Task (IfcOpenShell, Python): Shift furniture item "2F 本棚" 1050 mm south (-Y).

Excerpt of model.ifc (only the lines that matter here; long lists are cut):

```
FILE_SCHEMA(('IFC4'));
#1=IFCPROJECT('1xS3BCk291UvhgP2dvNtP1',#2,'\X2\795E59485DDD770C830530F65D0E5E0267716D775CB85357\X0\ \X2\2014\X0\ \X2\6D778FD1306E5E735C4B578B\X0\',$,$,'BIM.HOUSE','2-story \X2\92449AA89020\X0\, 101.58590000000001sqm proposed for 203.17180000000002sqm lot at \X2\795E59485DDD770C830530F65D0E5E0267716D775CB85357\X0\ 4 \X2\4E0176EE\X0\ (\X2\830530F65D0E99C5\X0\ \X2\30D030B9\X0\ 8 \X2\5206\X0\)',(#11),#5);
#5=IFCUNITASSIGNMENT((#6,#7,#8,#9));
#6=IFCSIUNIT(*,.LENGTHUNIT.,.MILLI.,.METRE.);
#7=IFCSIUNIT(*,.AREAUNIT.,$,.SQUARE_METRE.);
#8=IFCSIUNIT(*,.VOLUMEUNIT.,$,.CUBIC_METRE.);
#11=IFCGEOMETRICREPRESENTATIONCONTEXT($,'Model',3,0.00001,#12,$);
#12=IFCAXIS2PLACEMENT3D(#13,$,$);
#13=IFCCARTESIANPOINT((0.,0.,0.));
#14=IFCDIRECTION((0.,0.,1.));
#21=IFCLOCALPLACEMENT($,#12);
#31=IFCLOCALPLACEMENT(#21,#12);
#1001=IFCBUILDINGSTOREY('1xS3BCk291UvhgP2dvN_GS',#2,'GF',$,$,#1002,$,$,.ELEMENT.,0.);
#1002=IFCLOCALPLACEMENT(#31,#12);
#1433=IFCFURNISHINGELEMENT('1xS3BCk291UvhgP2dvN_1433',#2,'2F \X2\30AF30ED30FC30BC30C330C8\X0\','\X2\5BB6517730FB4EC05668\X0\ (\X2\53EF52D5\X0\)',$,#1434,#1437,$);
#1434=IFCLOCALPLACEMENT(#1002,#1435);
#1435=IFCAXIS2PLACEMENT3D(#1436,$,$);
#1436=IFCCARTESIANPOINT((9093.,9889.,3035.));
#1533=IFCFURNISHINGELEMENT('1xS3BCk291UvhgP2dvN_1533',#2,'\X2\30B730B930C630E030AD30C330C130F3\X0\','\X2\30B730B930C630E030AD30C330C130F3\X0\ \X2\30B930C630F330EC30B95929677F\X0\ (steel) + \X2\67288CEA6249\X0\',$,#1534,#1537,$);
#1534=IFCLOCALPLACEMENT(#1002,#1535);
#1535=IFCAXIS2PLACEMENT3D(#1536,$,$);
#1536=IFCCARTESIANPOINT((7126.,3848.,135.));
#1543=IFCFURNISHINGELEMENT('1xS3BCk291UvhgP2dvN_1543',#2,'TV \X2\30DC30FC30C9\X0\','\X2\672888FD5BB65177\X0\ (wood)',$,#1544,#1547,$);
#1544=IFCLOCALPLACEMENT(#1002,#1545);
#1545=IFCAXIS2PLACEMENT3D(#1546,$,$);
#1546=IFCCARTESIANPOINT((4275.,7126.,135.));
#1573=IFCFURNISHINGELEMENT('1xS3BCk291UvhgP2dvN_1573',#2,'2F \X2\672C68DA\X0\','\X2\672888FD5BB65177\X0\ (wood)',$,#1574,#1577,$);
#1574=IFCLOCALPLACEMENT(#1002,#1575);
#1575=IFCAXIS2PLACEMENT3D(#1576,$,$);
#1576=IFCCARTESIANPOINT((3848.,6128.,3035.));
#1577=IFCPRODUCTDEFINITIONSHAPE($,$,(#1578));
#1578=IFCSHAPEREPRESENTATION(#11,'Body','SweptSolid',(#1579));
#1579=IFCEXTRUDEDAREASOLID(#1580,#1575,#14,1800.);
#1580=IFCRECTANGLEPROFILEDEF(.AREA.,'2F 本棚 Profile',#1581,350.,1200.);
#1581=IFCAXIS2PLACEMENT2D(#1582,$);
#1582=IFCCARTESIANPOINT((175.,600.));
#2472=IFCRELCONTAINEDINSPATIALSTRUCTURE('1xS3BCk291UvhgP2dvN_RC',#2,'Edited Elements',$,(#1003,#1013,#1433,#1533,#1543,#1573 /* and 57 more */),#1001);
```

```python
import ifcopenshell
import ifcopenshell.api.geometry
import ifcopenshell.util.placement

model = ifcopenshell.open("model.ifc")

item = model.by_guid("1xS3BCk291UvhgP2dvN_1573")
matrix = ifcopenshell.util.placement.get_local_placement(item.ObjectPlacement)
matrix[1, 3] -= 1050.0
ifcopenshell.api.geometry.edit_object_placement(model, product=item, matrix=matrix, is_si=False)

print(ifcopenshell.util.placement.get_local_placement(item.ObjectPlacement).round(3) + 0.0)

model.write("model_v2.ifc")
```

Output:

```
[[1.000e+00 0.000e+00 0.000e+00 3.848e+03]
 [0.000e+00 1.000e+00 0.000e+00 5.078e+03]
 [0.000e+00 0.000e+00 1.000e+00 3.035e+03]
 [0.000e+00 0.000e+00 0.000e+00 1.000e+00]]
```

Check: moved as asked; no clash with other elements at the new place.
